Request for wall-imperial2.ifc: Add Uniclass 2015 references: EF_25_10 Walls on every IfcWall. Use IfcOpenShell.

First a look at what the model holds.

```python
import ifcopenshell

model = ifcopenshell.open("wall-imperial2.ifc")
print(model.schema)
print("classifications:", [c.Name for c in model.by_type("IfcClassification")])
for ifc_class in ("IfcDoor", "IfcRoof", "IfcStair", "IfcWall", "IfcWindow"):
    print(ifc_class, len(model.by_type(ifc_class)))
```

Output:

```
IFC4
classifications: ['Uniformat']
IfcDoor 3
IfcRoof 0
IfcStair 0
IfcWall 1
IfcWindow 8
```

```python
import ifcopenshell
import ifcopenshell.api.classification

model = ifcopenshell.open("wall-imperial2.ifc")

system = ifcopenshell.api.classification.add_classification(model, classification="Uniclass 2015")

codes = {
    "IfcWall": ("EF_25_10", "Walls"),
}
for ifc_class, (code, name) in codes.items():
    products = model.by_type(ifc_class)
    ifcopenshell.api.classification.add_reference(
        model, products=products, classification=system, identification=code, name=name
    )
    print(code, len(products))

model.write("wall-imperial2_updated.ifc")
```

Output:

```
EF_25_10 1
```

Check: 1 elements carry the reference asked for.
